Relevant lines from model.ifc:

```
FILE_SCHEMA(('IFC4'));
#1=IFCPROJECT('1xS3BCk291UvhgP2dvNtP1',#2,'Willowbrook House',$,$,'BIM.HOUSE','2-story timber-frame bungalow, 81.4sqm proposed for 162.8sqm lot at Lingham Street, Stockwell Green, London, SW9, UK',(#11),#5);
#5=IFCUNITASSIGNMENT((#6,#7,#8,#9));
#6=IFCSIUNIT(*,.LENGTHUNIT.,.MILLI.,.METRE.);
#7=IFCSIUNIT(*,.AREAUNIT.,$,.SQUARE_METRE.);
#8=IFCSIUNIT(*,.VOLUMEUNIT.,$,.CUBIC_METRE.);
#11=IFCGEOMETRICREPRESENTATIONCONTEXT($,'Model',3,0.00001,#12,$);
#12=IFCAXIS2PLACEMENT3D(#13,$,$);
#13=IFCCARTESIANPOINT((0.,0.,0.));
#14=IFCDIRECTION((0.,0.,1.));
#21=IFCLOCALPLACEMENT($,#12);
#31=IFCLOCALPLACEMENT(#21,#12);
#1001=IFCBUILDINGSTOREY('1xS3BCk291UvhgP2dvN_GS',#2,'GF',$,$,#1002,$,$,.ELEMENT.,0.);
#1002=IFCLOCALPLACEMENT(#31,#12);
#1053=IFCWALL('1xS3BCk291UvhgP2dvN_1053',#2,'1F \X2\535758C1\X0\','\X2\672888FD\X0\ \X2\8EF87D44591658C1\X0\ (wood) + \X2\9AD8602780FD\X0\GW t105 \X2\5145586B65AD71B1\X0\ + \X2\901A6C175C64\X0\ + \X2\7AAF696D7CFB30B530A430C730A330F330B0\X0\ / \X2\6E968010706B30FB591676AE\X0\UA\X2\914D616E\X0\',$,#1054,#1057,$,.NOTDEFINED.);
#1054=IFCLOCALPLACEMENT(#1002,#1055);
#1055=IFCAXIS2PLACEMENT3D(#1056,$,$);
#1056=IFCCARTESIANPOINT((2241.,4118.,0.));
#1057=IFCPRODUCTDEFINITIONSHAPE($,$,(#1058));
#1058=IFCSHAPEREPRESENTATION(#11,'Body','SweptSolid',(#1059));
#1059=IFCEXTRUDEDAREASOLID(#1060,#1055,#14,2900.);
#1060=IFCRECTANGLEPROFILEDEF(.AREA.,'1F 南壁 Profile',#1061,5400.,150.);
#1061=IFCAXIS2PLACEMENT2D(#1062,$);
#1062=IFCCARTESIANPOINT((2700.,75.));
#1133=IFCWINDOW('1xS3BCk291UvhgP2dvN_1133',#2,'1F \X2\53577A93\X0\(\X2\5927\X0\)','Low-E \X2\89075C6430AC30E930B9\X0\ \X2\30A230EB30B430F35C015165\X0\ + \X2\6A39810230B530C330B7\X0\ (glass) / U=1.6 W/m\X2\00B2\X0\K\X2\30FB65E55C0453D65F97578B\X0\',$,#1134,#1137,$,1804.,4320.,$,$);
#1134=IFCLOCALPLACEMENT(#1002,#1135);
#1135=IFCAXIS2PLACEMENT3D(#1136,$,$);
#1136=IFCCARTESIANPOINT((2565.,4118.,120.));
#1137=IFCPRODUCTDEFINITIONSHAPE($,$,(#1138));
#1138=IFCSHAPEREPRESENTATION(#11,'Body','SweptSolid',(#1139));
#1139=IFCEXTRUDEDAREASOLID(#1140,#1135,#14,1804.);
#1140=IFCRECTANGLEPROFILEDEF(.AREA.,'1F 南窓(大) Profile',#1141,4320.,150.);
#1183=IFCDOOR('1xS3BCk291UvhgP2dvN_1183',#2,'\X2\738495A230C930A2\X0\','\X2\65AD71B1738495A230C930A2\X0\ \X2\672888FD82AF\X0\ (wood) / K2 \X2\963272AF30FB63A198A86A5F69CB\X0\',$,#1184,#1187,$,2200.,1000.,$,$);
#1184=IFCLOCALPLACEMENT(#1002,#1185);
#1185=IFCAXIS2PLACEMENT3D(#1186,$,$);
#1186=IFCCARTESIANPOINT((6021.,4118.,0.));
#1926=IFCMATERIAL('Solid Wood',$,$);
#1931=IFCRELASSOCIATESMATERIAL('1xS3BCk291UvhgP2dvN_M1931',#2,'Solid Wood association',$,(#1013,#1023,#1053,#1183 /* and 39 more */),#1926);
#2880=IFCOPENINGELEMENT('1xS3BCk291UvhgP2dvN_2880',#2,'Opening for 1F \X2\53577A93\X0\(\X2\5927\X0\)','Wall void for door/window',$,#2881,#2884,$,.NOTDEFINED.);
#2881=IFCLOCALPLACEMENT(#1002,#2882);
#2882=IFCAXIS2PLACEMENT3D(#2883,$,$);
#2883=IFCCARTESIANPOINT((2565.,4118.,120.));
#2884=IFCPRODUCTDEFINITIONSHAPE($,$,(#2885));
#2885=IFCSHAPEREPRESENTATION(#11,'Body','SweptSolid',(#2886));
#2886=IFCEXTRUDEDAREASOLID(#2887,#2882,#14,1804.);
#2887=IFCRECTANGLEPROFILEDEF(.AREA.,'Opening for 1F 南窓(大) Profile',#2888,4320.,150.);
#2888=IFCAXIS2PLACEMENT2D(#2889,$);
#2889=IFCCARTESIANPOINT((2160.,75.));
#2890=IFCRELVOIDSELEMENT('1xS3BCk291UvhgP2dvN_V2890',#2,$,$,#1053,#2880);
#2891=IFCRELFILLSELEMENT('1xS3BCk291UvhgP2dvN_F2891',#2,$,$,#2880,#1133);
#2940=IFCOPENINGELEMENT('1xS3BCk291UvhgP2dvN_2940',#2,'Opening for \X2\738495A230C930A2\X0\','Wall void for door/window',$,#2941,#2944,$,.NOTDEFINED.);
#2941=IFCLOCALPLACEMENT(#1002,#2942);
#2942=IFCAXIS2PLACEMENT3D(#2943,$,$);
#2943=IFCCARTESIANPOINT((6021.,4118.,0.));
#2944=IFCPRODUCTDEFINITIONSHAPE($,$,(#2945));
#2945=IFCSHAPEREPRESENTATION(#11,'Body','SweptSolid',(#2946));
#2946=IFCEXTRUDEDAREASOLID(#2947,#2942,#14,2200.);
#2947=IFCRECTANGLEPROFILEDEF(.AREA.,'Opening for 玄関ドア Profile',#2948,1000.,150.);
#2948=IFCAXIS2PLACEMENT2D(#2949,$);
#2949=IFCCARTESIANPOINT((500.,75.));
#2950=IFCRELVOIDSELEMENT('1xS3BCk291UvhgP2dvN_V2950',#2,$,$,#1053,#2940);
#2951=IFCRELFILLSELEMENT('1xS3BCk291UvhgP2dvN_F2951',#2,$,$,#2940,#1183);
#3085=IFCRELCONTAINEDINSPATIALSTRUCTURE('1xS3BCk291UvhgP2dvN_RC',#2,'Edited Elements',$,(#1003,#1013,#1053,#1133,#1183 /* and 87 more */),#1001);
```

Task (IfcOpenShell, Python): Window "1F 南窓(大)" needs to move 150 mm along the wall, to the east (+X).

```python
import ifcopenshell
import ifcopenshell.api.geometry
import ifcopenshell.util.placement

model = ifcopenshell.open("model.ifc")

window = model.by_guid("1xS3BCk291UvhgP2dvN_1133")
opening = window.FillsVoids[0].RelatingOpeningElement
wall = opening.VoidsElements[0].RelatingBuildingElement

wall_matrix = ifcopenshell.util.placement.get_local_placement(wall.ObjectPlacement)
shift = wall_matrix[:3, 0] * 150.0
before = ifcopenshell.util.placement.get_local_placement(window.ObjectPlacement)[:3, 3].copy()

# The window is not placed relative to its opening, so move both.
for product in (opening, window):
    matrix = ifcopenshell.util.placement.get_local_placement(product.ObjectPlacement)
    matrix[:3, 3] += shift
    ifcopenshell.api.geometry.edit_object_placement(model, product=product, matrix=matrix, is_si=False)

after = ifcopenshell.util.placement.get_local_placement(window.ObjectPlacement)[:3, 3]
print("window moved by", (after - before).round(3) + 0.0)

model.write("model_v2.ifc")
```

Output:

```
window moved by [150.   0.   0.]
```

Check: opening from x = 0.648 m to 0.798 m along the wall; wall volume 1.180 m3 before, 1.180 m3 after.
